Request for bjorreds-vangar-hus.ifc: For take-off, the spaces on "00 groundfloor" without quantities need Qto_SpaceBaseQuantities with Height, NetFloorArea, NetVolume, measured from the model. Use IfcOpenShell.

First a look at what the model holds.

```python
import ifcopenshell
import ifcopenshell.util.element
import ifcopenshell.util.unit

model = ifcopenshell.open("bjorreds-vangar-hus.ifc")
print(model.schema)
for unit_type in ("LENGTHUNIT", "AREAUNIT", "VOLUMEUNIT"):
    print(unit_type, ifcopenshell.util.unit.calculate_unit_scale(model, unit_type))
storey = next(s for s in model.by_type("IfcBuildingStorey") if s.Name == "00 groundfloor")
spaces = [e for e in ifcopenshell.util.element.get_decomposition(storey) if e.is_a("IfcSpace")]
for e in sorted(spaces, key=lambda e: e.id()):
    print(e.id(), e.is_a(), e.Name, list(ifcopenshell.util.element.get_psets(e, qtos_only=True)), sep=" | ")
```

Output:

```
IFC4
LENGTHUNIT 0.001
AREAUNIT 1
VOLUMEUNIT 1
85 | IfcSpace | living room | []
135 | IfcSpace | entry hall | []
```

```python
import ifcopenshell
import ifcopenshell.api.pset
import ifcopenshell.geom
import ifcopenshell.util.element
import ifcopenshell.util.shape
import ifcopenshell.util.unit

model = ifcopenshell.open("bjorreds-vangar-hus.ifc")
unit_scale = ifcopenshell.util.unit.calculate_unit_scale(model)
area_scale = ifcopenshell.util.unit.calculate_unit_scale(model, "AREAUNIT")
volume_scale = ifcopenshell.util.unit.calculate_unit_scale(model, "VOLUMEUNIT")
settings = ifcopenshell.geom.settings()

storey = next(s for s in model.by_type("IfcBuildingStorey") if s.Name == "00 groundfloor")
spaces = [e for e in ifcopenshell.util.element.get_decomposition(storey) if e.is_a("IfcSpace")]

for e in sorted(spaces, key=lambda e: e.id()):
    if ifcopenshell.util.element.get_psets(e, qtos_only=True, should_inherit=False):
        continue
    # Geometry comes back in metres, in the element's own axes.
    shape = ifcopenshell.geom.create_shape(settings, e)
    values = {
        "Height": ifcopenshell.util.shape.get_z(shape.geometry) / unit_scale,
        "NetFloorArea": ifcopenshell.util.shape.get_footprint_area(shape.geometry) / area_scale,
        "NetVolume": ifcopenshell.util.shape.get_volume(shape.geometry) / volume_scale,
    }
    qto = ifcopenshell.api.pset.add_qto(model, product=e, name="Qto_SpaceBaseQuantities")
    ifcopenshell.api.pset.edit_qto(model, qto=qto, properties=values)
    print(e.id(), {k: round(v, 3) for k, v in values.items()})

model.write("bjorreds-vangar-hus_edited.ifc")
```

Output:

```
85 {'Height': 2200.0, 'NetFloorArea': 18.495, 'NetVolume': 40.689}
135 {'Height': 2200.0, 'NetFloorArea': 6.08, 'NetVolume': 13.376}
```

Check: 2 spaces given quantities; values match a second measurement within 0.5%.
